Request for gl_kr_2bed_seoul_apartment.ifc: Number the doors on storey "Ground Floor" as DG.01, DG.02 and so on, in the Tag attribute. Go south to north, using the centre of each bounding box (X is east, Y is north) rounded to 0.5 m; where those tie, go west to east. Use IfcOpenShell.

First a look at what the model holds.

```python
import ifcopenshell
import ifcopenshell.util.element
import ifcopenshell.util.placement

model = ifcopenshell.open("gl_kr_2bed_seoul_apartment.ifc")
print(model.schema)
storey = next(s for s in model.by_type("IfcBuildingStorey") if s.Name == "Ground Floor")
doors = [e for e in ifcopenshell.util.element.get_decomposition(storey) if e.is_a("IfcDoor")]
for e in sorted(doors, key=lambda e: e.id()):
    origin = ifcopenshell.util.placement.get_local_placement(e.ObjectPlacement)[:3, 3]
    print(e.id(), e.Tag, e.Name, origin.round(2) + 0.0, sep=" | ")
```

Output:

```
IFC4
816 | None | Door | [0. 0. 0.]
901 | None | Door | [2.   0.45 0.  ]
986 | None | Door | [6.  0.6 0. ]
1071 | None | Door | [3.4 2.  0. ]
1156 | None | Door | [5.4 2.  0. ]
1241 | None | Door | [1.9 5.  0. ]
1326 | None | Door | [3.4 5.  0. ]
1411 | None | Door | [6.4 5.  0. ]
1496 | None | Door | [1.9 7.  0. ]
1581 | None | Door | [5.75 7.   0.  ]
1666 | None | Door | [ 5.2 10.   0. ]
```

```python
import ifcopenshell
import ifcopenshell.geom
import ifcopenshell.util.element
import ifcopenshell.util.shape

model = ifcopenshell.open("gl_kr_2bed_seoul_apartment.ifc")
settings = ifcopenshell.geom.settings()
settings.set("use-world-coords", True)


def centre(element):
    shape = ifcopenshell.geom.create_shape(settings, element)
    return ifcopenshell.util.shape.get_bbox_centroid(shape.geometry)


storey = next(s for s in model.by_type("IfcBuildingStorey") if s.Name == "Ground Floor")
doors = [e for e in ifcopenshell.util.element.get_decomposition(storey) if e.is_a("IfcDoor")]

# Insertion points can sit at a corner or the storey origin, so sort by the geometry (in metres).
centres = {e: centre(e) for e in doors}
doors.sort(key=lambda e: (round(centres[e][1] / 0.5), centres[e][0]))

for i, e in enumerate(doors, start=1):
    number = f"DG.{i:02d}"
    e.Tag = number
    print(e.id(), number)

model.write("gl_kr_2bed_seoul_apartment_v2.ifc")
```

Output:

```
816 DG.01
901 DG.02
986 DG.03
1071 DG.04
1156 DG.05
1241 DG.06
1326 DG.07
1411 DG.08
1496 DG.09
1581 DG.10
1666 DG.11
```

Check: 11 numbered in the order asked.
